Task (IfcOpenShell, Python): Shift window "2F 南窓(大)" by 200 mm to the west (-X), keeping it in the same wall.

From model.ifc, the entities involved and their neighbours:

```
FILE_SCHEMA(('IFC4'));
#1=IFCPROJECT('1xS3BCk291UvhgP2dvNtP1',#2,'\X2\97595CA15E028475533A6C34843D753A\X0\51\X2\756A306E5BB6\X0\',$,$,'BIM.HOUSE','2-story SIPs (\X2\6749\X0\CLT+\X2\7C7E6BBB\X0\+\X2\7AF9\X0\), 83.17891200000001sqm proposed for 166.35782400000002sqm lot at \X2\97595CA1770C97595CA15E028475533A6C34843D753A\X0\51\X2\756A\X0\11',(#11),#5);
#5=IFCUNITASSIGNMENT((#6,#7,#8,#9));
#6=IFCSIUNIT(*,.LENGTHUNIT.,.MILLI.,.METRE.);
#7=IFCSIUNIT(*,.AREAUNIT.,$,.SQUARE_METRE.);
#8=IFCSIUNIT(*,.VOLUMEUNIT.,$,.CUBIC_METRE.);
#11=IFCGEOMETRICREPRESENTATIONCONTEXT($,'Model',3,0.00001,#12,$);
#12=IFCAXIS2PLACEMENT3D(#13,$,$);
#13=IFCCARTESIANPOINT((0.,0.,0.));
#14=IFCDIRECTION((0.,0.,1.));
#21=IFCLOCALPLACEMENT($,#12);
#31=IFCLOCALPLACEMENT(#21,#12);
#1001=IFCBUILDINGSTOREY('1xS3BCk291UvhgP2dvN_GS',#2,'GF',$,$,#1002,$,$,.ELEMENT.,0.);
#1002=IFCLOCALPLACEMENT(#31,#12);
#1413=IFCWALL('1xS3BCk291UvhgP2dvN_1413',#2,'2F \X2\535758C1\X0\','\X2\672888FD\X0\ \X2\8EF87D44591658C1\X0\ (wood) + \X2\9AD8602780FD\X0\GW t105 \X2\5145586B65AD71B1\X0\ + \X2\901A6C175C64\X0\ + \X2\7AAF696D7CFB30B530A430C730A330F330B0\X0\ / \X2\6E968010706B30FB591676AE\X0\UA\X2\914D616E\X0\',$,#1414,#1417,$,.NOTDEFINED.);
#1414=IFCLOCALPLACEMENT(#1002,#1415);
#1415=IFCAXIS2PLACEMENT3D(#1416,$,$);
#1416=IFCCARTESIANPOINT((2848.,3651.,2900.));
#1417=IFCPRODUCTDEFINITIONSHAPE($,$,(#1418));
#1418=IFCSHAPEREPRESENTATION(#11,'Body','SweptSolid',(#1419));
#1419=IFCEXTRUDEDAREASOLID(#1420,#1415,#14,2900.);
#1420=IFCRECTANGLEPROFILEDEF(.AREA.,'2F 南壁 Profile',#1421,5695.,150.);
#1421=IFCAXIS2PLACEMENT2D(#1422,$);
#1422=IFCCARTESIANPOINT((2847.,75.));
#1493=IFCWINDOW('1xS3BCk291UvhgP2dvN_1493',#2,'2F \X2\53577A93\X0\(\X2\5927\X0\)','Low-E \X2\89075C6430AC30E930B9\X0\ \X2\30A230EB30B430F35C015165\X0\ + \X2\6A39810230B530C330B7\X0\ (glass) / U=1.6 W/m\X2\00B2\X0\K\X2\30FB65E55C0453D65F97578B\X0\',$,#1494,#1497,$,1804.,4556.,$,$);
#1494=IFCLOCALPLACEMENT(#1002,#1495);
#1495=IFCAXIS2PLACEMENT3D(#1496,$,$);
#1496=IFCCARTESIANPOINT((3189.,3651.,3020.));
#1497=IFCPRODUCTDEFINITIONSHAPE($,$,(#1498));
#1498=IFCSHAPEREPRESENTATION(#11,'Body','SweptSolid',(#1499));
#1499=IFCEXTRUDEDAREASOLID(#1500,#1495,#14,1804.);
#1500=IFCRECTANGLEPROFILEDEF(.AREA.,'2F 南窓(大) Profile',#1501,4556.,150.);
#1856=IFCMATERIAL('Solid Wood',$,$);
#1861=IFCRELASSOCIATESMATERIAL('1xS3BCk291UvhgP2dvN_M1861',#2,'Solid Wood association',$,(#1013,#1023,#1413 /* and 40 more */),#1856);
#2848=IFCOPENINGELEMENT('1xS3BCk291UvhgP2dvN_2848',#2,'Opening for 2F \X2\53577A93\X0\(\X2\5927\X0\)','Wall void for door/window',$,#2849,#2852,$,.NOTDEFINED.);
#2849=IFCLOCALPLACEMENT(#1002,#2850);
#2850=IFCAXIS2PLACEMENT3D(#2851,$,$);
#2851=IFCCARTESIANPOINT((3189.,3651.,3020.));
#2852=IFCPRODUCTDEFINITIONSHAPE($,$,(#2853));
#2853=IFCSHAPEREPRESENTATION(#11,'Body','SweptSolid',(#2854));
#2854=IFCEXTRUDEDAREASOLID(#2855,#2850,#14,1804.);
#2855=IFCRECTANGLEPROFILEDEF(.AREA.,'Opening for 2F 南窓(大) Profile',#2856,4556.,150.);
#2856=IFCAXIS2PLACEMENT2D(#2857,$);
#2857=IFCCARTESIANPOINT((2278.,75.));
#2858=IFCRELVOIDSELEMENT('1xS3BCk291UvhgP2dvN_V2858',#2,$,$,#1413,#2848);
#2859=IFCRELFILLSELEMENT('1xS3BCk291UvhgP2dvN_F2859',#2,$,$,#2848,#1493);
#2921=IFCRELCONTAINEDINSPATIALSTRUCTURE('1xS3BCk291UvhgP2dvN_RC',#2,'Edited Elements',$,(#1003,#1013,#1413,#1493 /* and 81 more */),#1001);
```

```python
import ifcopenshell
import ifcopenshell.api.geometry
import ifcopenshell.util.placement

model = ifcopenshell.open("model.ifc")

window = model.by_id(1493)
opening = window.FillsVoids[0].RelatingOpeningElement
wall = opening.VoidsElements[0].RelatingBuildingElement

wall_matrix = ifcopenshell.util.placement.get_local_placement(wall.ObjectPlacement)
shift = wall_matrix[:3, 0] * -200.0
before = ifcopenshell.util.placement.get_local_placement(window.ObjectPlacement)[:3, 3].copy()

# The window is not placed relative to its opening, so move both.
for product in (opening, window):
    matrix = ifcopenshell.util.placement.get_local_placement(product.ObjectPlacement)
    matrix[:3, 3] += shift
    ifcopenshell.api.geometry.edit_object_placement(model, product=product, matrix=matrix, is_si=False)

after = ifcopenshell.util.placement.get_local_placement(window.ObjectPlacement)[:3, 3]
print("window moved by", (after - before).round(3) + 0.0)

model.write("model-out.ifc")
```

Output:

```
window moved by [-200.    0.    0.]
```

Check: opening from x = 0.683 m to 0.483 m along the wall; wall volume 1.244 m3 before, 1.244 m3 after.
